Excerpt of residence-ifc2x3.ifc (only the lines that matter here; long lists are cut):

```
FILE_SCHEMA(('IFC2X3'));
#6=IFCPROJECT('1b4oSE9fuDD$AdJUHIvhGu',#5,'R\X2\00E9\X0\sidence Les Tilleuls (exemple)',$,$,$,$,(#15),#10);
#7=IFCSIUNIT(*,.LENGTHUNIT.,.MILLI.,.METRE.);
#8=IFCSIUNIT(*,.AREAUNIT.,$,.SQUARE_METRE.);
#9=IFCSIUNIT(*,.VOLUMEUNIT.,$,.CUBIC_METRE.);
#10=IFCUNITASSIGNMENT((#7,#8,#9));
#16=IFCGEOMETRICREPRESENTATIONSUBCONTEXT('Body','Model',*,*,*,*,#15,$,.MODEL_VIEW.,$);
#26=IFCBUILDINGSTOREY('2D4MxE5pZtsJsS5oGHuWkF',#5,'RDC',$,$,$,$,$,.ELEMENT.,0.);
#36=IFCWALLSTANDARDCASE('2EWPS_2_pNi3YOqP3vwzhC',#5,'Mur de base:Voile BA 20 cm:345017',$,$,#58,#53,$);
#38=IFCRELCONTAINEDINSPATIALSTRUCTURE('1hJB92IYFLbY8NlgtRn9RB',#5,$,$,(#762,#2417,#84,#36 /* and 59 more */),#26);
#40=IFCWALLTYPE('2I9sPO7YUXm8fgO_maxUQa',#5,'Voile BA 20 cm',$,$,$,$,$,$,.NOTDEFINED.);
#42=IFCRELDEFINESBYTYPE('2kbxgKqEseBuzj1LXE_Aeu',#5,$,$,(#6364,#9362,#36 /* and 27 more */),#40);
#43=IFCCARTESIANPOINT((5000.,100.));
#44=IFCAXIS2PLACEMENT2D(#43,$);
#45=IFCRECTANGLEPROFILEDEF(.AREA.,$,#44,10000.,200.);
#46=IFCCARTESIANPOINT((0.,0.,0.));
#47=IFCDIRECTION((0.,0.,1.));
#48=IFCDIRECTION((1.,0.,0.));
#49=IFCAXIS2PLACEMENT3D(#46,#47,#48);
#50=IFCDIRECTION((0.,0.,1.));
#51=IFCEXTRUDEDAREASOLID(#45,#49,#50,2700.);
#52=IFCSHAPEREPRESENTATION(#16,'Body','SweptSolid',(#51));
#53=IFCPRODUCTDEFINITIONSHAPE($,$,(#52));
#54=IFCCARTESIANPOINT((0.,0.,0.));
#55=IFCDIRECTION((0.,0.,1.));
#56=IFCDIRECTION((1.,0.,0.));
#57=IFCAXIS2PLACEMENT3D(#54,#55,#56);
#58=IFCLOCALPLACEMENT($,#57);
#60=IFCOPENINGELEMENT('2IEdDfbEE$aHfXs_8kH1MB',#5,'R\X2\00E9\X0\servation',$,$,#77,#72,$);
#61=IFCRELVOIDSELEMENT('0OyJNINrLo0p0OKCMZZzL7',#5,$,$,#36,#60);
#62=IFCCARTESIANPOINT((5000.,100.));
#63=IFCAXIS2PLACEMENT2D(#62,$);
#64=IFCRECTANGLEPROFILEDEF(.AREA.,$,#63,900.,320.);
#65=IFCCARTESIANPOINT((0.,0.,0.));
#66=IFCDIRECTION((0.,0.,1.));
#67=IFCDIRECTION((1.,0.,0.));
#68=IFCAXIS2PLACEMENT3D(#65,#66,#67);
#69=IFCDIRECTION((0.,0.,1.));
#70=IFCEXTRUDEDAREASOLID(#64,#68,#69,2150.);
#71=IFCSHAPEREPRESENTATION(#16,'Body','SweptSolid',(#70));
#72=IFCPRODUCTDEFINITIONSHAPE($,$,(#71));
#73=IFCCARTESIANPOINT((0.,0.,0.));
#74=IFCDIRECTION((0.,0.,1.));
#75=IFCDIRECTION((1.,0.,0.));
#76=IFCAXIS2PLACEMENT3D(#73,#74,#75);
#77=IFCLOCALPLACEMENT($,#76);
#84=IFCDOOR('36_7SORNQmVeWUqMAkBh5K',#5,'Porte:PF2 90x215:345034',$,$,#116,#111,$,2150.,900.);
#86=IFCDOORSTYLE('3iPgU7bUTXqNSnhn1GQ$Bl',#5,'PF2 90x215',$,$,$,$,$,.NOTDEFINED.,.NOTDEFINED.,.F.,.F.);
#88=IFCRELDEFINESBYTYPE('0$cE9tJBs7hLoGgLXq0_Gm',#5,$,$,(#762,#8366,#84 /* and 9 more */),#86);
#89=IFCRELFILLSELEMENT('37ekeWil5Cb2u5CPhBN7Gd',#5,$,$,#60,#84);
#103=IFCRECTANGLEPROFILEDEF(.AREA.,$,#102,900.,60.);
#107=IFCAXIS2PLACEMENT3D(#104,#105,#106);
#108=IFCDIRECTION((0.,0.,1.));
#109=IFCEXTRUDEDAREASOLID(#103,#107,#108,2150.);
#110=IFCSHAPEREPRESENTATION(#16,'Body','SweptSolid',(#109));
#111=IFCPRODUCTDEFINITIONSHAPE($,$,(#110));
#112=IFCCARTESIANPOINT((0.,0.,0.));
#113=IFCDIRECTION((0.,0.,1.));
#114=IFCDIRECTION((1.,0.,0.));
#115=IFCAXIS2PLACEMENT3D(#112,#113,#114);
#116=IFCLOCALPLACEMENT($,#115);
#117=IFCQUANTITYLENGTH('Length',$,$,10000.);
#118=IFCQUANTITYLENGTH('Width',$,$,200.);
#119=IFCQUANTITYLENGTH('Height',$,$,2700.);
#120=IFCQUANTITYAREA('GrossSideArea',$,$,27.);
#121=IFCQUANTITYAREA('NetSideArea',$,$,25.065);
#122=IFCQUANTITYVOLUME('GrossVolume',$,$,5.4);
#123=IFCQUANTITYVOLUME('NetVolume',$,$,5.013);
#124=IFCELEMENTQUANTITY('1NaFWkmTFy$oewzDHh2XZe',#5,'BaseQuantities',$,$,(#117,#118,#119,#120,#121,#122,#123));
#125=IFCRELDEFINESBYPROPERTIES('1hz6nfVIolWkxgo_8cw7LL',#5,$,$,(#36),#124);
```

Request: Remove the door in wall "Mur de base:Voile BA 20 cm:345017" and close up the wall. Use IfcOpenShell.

```python
import ifcopenshell
import ifcopenshell.api.feature
import ifcopenshell.api.pset
import ifcopenshell.api.root
import ifcopenshell.geom
import ifcopenshell.util.element
import ifcopenshell.util.shape
import ifcopenshell.util.unit

model = ifcopenshell.open("residence-ifc2x3.ifc")
area_scale = ifcopenshell.util.unit.calculate_unit_scale(model, "AREAUNIT")
volume_scale = ifcopenshell.util.unit.calculate_unit_scale(model, "VOLUMEUNIT")
settings = ifcopenshell.geom.settings()


def volume(element):
    """Net volume in cubic metres, openings subtracted."""
    shape = ifcopenshell.geom.create_shape(settings, element)
    return ifcopenshell.util.shape.get_volume(shape.geometry)


door = model.by_id(84)
opening = door.FillsVoids[0].RelatingOpeningElement
wall = opening.VoidsElements[0].RelatingBuildingElement
before = volume(wall)

ifcopenshell.api.root.remove_product(model, product=door)
ifcopenshell.api.feature.remove_feature(model, feature=opening)

after = volume(wall)
thickness = 0.2  # wall thickness in metres

# Update the wall's stored quantities.
qto = model.by_id(ifcopenshell.util.element.get_pset(wall, "BaseQuantities", should_inherit=False)["id"])
ifcopenshell.api.pset.edit_qto(model, qto=qto, properties={
    "NetSideArea": after / thickness / area_scale,
    "NetVolume": after / volume_scale,
})

print(f"wall volume {before:.3f} -> {after:.3f} m3")

model.write("residence-ifc2x3_v2.ifc")
```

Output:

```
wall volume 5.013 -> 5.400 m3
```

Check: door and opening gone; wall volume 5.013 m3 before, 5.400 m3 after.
